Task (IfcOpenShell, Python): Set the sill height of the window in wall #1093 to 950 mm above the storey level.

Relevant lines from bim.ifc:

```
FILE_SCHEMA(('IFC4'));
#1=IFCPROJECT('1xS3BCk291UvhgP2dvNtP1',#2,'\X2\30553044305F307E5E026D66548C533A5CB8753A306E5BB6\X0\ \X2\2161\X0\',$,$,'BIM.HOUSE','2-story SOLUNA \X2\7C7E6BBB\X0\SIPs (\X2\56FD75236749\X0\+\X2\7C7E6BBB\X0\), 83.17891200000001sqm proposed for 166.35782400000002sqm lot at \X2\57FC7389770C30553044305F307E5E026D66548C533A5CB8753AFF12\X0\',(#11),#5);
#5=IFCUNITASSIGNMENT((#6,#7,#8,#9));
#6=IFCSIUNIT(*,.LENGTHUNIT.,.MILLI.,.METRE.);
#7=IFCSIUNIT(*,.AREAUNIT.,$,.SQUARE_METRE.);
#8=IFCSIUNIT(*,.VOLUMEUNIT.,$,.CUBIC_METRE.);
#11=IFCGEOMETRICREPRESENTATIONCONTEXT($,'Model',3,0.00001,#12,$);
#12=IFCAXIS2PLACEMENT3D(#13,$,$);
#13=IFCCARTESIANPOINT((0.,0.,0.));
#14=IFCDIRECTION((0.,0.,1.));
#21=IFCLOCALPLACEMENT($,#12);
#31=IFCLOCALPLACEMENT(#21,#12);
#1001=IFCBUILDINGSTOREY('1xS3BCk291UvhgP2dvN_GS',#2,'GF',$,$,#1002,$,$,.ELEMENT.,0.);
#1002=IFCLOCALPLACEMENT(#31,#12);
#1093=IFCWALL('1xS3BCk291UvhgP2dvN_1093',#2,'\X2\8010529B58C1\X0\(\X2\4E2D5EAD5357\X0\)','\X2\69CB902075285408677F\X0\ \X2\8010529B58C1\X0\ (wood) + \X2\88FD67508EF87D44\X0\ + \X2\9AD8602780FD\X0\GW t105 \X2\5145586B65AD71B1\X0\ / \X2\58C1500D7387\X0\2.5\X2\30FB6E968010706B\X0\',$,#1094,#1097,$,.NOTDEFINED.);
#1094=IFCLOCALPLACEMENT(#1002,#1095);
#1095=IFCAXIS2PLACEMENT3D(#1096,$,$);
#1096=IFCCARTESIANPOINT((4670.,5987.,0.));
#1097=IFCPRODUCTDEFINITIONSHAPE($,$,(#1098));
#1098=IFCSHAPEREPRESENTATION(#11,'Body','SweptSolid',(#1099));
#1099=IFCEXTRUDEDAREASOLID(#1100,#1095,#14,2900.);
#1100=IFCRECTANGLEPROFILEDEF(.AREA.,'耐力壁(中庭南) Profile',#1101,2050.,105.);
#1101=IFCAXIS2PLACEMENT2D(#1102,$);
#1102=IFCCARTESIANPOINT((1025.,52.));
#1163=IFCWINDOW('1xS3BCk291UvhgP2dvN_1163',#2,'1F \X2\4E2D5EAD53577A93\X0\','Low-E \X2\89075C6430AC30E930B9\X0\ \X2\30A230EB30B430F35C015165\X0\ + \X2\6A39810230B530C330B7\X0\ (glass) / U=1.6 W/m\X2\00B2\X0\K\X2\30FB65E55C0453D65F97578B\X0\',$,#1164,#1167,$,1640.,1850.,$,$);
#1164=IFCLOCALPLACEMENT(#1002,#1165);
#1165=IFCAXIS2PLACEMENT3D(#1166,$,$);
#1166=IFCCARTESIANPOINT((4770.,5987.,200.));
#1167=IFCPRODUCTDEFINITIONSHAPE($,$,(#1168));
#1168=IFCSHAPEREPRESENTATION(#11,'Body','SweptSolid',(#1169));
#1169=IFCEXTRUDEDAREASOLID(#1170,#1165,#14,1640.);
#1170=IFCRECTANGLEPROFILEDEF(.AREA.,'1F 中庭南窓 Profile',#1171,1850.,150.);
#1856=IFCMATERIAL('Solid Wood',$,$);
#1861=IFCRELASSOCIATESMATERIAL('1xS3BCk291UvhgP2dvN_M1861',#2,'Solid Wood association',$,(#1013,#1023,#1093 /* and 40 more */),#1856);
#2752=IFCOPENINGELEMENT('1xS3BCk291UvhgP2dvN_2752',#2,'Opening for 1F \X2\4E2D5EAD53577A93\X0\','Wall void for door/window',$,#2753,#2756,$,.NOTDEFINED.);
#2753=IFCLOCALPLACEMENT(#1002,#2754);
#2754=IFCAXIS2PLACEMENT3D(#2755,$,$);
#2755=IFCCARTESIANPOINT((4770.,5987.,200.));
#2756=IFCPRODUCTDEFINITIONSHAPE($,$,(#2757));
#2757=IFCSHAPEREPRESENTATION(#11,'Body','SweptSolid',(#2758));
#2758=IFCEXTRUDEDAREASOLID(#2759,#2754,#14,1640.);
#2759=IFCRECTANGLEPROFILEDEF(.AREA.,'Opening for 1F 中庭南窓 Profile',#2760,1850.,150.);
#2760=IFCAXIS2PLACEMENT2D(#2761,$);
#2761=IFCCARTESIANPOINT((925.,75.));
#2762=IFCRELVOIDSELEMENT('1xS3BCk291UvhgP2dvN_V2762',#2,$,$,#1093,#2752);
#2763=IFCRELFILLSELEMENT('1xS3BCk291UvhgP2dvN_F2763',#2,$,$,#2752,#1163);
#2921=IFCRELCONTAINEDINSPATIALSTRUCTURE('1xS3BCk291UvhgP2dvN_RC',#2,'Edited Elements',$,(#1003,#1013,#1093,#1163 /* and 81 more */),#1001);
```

```python
import numpy as np
import ifcopenshell
import ifcopenshell.api.geometry
import ifcopenshell.geom
import ifcopenshell.util.element
import ifcopenshell.util.placement
import ifcopenshell.util.shape
import ifcopenshell.util.unit

model = ifcopenshell.open("bim.ifc")
unit_scale = ifcopenshell.util.unit.calculate_unit_scale(model)

window = model.by_guid("1xS3BCk291UvhgP2dvN_1163")
opening = window.FillsVoids[0].RelatingOpeningElement
storey = ifcopenshell.util.element.get_container(window, ifc_class="IfcBuildingStorey")
level = ifcopenshell.util.placement.get_local_placement(storey.ObjectPlacement)[2, 3]

# The opening's origin need not be at the sill, so measure its lowest point.
shape = ifcopenshell.geom.create_shape(ifcopenshell.geom.settings(), opening)
bottom = ifcopenshell.util.shape.get_shape_bottom_elevation(shape, shape.geometry) / unit_scale
dz = level + 0.95 / unit_scale - bottom

shift = np.array([0.0, 0.0, dz])
# The window is not placed relative to its opening, so move both.
for product in (opening, window):
    matrix = ifcopenshell.util.placement.get_local_placement(product.ObjectPlacement)
    matrix[:3, 3] += shift
    ifcopenshell.api.geometry.edit_object_placement(model, product=product, matrix=matrix, is_si=False)

print(f"moved by {dz * unit_scale:+.3f} m")

model.write("bim_rev.ifc")
```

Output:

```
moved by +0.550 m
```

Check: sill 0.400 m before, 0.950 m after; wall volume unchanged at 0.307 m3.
